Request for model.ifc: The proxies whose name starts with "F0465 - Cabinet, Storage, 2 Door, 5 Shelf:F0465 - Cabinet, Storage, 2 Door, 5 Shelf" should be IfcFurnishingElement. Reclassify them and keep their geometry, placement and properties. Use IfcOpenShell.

First a look at what the model holds.

```python
import re

import ifcopenshell

model = ifcopenshell.open("model.ifc")
print(model.schema)
seen = {}
for e in model.by_type("IfcBuildingElementProxy"):
    name = re.sub(r":\d+(:\d+)?$", "", e.Name or "")  # drop the element id that some exporters append
    seen[name] = seen.get(name, 0) + 1
for name, count in sorted(seen.items()):
    print(count, "x", name)
```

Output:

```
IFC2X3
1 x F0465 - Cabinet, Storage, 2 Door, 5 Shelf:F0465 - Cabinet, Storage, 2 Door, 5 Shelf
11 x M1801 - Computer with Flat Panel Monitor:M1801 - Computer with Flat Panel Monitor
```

```python
import ifcopenshell
import ifcopenshell.api.root

model = ifcopenshell.open("model.ifc")

proxies = [e.id() for e in model.by_type("IfcBuildingElementProxy") if (e.Name or "").startswith("F0465 - Cabinet, Storage, 2 Door, 5 Shelf:F0465 - Cabinet, Storage, 2 Door, 5 Shelf")]
for step_id in proxies:
    proxy = model.by_id(step_id)
    # Reclassifying a typed element also reclassifies its type and the type's other occurrences.
    if proxy.is_a("IfcBuildingElementProxy"):
        ifcopenshell.api.root.reassign_class(model, product=proxy, ifc_class="IfcFurnishingElement")

print(sum(model.by_id(i).is_a("IfcFurnishingElement") for i in proxies), "reclassified")

model.write("model_edited.ifc")
```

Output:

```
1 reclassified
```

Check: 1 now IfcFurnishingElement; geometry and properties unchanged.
